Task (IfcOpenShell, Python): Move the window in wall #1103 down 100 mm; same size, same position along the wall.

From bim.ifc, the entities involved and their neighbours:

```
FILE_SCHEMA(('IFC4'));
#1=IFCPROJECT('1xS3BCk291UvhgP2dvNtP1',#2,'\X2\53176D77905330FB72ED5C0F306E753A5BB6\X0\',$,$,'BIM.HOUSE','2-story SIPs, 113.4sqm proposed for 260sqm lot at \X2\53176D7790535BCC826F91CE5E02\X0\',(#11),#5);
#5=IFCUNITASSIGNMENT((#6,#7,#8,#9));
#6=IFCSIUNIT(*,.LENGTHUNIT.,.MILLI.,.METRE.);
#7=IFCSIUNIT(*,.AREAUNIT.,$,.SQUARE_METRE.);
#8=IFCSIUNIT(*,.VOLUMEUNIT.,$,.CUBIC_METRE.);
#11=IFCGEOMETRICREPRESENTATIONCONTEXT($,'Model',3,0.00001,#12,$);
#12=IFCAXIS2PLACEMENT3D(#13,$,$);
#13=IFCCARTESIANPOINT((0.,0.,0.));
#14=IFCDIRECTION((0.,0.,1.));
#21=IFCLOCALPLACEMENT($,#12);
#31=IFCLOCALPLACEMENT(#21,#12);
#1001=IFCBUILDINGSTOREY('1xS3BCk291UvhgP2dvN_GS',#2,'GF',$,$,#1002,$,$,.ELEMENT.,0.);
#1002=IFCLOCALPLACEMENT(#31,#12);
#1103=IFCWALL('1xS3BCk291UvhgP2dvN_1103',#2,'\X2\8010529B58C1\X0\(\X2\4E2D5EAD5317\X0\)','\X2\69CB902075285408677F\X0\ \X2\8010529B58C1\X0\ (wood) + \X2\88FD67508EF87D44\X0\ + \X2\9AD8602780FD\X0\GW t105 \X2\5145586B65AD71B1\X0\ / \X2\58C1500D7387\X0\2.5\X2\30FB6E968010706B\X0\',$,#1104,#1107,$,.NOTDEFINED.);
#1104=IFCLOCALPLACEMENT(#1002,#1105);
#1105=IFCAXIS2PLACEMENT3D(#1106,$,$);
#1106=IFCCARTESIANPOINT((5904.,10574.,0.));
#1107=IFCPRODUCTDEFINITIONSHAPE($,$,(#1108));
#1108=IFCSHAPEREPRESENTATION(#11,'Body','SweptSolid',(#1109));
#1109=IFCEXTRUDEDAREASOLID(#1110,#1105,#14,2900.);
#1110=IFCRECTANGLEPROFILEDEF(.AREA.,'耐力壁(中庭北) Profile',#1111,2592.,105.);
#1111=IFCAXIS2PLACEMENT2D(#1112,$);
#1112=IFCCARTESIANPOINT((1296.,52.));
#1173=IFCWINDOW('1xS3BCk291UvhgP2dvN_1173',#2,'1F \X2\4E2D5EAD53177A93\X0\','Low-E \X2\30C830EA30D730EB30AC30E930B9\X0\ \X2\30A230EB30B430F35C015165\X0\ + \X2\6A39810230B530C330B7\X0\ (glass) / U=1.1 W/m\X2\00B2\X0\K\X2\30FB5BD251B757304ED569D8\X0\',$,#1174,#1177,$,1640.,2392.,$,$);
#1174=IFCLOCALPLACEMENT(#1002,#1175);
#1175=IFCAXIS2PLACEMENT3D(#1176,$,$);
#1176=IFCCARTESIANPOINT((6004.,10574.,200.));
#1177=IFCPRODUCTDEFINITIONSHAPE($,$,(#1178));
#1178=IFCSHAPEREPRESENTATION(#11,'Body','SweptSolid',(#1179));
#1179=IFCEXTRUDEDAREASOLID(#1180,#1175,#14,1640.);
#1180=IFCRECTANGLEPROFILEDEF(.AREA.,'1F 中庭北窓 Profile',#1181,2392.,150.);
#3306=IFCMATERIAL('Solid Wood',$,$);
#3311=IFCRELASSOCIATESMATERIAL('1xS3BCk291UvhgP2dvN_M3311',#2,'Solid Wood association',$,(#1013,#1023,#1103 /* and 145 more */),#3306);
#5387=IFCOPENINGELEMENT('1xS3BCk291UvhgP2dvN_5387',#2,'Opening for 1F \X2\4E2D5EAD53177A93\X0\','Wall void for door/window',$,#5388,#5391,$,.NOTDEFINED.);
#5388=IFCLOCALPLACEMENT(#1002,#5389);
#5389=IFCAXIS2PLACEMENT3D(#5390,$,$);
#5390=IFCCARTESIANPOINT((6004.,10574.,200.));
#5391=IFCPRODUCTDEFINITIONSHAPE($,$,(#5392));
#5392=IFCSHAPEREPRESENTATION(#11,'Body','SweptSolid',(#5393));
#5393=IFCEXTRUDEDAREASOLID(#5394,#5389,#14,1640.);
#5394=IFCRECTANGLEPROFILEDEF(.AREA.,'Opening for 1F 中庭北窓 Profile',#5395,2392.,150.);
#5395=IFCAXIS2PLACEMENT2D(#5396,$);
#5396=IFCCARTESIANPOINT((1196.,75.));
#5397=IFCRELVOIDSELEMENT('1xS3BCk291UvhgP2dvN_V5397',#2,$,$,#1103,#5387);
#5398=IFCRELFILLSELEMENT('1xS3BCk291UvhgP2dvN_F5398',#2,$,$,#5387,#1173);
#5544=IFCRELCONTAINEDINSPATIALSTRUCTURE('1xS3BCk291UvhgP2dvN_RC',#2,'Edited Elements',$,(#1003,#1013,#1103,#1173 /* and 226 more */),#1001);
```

```python
import numpy as np
import ifcopenshell
import ifcopenshell.api.geometry
import ifcopenshell.util.placement
import ifcopenshell.util.unit

model = ifcopenshell.open("bim.ifc")
unit_scale = ifcopenshell.util.unit.calculate_unit_scale(model)

window = model.by_id(1173)
opening = window.FillsVoids[0].RelatingOpeningElement
dz = -0.1 / unit_scale

shift = np.array([0.0, 0.0, dz])
# The window is not placed relative to its opening, so move both.
for product in (opening, window):
    matrix = ifcopenshell.util.placement.get_local_placement(product.ObjectPlacement)
    matrix[:3, 3] += shift
    ifcopenshell.api.geometry.edit_object_placement(model, product=product, matrix=matrix, is_si=False)

print(f"moved by {dz * unit_scale:+.3f} m")

model.write("bim_edited.ifc")
```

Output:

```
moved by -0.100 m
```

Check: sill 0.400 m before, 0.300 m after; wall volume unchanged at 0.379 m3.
